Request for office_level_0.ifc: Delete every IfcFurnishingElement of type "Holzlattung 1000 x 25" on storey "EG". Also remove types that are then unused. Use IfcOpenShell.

First a look at what the model holds.

```python
import ifcopenshell
import ifcopenshell.util.element

model = ifcopenshell.open("office_level_0.ifc")
print(model.schema)
storey = next(s for s in model.by_type("IfcBuildingStorey") if s.Name == "EG")
furniture = [e for e in ifcopenshell.util.element.get_decomposition(storey) if e.is_a("IfcFurnishingElement")]
seen = {}
for e in furniture:
    element_type = ifcopenshell.util.element.get_type(e)
    name = element_type.Name if element_type not in (None, e) else None
    seen[name] = seen.get(name, 0) + 1
for name, count in sorted(seen.items(), key=str):
    print(count, "x", name)
```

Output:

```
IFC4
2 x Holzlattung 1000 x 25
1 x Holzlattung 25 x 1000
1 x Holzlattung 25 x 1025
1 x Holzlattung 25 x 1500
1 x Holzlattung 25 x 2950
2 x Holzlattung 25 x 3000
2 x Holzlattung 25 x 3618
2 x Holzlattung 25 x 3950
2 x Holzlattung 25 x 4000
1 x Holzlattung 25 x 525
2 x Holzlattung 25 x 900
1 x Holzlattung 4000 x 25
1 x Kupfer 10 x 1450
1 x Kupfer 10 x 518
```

```python
import ifcopenshell
import ifcopenshell.api.root
import ifcopenshell.util.element

model = ifcopenshell.open("office_level_0.ifc")

storey = next(s for s in model.by_type("IfcBuildingStorey") if s.Name == "EG")
furniture = [e for e in ifcopenshell.util.element.get_decomposition(storey) if e.is_a("IfcFurnishingElement")]
targets = [e for e in furniture if (t := ifcopenshell.util.element.get_type(e)) not in (None, e) and t.Name == "Holzlattung 1000 x 25"]
types = {ifcopenshell.util.element.get_type(e) for e in targets} - {None, *targets}

for e in targets:
    ifcopenshell.api.root.remove_product(model, product=e)
print(len(targets), "removed")

unused = [t for t in types if not ifcopenshell.util.element.get_types(t)]
for t in unused:
    ifcopenshell.api.root.remove_product(model, product=t)
print(len(unused), "unused types removed")

model.write("office_level_0_rev.ifc")
```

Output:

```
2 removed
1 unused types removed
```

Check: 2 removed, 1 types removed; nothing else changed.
